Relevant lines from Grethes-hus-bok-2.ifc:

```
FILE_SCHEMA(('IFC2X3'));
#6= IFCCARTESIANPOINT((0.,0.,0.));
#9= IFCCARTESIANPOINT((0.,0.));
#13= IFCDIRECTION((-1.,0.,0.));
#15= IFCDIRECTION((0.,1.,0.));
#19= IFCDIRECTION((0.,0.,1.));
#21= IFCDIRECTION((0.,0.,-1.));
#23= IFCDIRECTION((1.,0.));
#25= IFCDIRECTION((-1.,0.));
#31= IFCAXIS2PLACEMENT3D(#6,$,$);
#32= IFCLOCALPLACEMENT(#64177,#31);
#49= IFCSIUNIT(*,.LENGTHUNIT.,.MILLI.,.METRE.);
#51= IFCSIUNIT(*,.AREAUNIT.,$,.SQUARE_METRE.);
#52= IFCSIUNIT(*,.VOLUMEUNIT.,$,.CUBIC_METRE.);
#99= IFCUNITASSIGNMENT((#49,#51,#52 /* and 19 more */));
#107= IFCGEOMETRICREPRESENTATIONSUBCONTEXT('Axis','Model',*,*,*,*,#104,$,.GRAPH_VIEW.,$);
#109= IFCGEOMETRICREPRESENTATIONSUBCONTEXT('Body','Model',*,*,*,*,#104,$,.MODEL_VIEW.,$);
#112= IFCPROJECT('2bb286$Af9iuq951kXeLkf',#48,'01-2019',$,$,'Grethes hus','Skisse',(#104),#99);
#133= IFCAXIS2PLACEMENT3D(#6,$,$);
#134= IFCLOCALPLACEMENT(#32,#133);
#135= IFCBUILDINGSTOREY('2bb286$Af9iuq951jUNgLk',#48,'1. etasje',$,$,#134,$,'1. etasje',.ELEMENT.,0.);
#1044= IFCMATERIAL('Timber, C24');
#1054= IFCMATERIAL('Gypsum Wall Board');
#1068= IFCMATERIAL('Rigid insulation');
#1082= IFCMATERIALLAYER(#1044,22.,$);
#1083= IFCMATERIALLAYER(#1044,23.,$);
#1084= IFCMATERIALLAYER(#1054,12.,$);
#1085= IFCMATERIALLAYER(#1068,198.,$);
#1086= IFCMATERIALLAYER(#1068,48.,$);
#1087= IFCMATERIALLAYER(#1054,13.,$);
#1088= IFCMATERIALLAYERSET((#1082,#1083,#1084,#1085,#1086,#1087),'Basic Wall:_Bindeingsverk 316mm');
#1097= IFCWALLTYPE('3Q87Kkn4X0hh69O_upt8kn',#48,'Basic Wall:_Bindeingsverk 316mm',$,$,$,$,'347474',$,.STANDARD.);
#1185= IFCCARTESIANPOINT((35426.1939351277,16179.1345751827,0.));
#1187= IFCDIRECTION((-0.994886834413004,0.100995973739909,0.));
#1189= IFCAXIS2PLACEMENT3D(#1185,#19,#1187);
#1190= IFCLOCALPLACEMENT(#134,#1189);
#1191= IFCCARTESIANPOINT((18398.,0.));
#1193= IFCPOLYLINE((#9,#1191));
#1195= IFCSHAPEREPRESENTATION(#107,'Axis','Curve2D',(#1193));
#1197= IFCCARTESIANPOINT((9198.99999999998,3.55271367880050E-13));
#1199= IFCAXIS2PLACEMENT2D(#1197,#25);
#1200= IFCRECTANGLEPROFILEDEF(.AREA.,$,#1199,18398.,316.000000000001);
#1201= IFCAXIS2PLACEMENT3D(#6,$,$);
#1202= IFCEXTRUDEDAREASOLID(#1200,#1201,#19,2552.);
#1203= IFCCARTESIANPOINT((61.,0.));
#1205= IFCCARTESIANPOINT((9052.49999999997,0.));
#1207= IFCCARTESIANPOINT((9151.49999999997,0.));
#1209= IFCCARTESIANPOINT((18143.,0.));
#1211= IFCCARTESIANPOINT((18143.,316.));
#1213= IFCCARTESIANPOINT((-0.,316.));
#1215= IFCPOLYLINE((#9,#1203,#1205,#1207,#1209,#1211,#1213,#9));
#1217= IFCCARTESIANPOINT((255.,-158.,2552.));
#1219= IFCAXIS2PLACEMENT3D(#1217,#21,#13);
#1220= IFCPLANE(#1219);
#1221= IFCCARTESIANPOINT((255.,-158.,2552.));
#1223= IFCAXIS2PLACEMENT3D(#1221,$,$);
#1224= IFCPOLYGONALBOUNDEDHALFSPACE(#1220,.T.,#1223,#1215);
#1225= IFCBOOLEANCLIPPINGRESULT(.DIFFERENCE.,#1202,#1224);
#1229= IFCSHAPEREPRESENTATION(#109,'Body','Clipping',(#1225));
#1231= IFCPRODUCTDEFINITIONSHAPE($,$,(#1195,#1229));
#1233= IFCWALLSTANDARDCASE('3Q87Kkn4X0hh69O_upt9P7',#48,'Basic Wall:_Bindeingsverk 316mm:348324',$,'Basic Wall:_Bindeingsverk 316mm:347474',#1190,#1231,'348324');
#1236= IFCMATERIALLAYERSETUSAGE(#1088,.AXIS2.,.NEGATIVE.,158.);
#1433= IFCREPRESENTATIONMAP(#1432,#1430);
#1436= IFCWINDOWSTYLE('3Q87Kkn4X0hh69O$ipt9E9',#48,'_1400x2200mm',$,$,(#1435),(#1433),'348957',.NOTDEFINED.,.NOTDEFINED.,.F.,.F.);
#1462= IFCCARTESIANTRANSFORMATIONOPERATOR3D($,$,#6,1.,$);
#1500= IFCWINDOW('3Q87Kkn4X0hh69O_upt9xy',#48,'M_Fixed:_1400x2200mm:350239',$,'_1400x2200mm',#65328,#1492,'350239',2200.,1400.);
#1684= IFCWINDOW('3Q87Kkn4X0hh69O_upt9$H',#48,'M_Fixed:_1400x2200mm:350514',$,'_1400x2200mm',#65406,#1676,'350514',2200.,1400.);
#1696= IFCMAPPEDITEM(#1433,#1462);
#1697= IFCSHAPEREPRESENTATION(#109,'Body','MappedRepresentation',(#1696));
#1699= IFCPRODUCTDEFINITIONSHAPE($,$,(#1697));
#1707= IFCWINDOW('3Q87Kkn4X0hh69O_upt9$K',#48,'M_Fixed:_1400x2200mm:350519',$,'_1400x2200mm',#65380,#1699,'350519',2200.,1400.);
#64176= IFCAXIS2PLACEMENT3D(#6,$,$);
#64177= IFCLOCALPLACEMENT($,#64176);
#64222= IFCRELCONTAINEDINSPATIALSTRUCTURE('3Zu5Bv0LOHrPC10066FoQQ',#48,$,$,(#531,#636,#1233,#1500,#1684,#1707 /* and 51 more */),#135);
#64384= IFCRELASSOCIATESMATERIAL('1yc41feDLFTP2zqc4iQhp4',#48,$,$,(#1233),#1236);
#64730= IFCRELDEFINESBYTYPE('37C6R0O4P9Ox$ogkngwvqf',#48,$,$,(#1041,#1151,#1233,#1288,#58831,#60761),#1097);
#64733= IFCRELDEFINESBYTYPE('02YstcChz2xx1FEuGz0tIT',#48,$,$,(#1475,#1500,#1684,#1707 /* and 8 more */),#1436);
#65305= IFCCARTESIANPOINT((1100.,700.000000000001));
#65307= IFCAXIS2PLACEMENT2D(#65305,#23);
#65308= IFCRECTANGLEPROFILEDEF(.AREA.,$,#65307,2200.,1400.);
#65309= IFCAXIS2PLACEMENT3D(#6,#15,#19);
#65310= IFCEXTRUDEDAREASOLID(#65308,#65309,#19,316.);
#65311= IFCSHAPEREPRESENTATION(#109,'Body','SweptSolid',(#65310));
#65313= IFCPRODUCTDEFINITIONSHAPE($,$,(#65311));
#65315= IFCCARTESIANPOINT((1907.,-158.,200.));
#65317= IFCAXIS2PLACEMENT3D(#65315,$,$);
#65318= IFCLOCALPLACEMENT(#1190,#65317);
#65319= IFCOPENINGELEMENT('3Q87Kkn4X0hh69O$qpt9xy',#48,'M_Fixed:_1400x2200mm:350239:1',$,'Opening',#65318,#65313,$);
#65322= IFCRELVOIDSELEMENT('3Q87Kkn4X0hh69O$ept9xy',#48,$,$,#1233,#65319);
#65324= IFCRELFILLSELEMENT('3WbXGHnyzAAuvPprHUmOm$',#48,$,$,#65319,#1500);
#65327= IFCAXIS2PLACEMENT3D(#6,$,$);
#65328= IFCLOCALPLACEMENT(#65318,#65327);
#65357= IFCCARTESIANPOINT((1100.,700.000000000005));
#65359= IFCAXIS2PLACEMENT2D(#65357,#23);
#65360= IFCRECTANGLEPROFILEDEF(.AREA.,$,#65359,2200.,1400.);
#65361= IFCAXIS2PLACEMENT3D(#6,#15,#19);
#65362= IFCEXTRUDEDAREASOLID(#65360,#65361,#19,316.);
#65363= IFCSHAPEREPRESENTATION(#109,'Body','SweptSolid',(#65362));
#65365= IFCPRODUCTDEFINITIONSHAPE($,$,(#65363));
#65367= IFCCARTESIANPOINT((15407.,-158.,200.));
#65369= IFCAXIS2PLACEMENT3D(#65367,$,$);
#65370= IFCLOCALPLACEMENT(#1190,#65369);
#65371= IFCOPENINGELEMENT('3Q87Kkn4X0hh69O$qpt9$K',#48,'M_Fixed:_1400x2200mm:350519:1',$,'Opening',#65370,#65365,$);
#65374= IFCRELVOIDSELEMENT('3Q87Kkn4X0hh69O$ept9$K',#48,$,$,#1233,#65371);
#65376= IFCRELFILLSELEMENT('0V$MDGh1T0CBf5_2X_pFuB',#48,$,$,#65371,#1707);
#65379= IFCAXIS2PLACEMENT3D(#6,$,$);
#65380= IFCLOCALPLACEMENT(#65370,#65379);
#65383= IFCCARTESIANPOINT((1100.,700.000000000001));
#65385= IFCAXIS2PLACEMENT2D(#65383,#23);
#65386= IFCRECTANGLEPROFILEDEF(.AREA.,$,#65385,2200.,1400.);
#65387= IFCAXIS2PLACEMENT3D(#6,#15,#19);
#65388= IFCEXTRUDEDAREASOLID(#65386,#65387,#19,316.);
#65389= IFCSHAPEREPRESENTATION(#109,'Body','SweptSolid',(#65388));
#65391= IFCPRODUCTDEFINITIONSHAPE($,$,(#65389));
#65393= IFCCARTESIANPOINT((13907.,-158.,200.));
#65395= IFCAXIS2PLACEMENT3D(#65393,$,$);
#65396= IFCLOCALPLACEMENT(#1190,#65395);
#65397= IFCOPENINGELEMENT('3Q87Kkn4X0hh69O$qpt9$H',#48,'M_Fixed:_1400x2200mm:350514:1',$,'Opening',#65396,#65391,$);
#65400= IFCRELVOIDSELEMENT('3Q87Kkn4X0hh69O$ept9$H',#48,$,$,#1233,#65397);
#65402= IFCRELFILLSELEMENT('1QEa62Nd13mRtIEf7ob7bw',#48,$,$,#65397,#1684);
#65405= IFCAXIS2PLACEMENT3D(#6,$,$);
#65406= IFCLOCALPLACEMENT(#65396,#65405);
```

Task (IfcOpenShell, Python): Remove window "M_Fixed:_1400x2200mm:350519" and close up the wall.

```python
import ifcopenshell
import ifcopenshell.api.feature
import ifcopenshell.api.root
import ifcopenshell.geom
import ifcopenshell.util.shape

model = ifcopenshell.open("Grethes-hus-bok-2.ifc")
settings = ifcopenshell.geom.settings()


def volume(element):
    """Net volume in cubic metres, openings subtracted."""
    shape = ifcopenshell.geom.create_shape(settings, element)
    return ifcopenshell.util.shape.get_volume(shape.geometry)


window = model.by_id(1707)
opening = window.FillsVoids[0].RelatingOpeningElement
wall = opening.VoidsElements[0].RelatingBuildingElement
before = volume(wall)

ifcopenshell.api.root.remove_product(model, product=window)
ifcopenshell.api.feature.remove_feature(model, feature=opening)

after = volume(wall)

print(f"wall volume {before:.3f} -> {after:.3f} m3")

model.write("Grethes-hus-bok-2-out.ifc")
```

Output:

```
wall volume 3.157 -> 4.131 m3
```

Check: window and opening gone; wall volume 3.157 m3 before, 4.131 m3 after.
